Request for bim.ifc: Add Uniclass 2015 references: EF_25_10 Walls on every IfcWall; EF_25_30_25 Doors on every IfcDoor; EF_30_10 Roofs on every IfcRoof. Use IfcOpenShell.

First a look at what the model holds.

```python
import ifcopenshell

model = ifcopenshell.open("bim.ifc")
print(model.schema)
print("classifications:", [c.Name for c in model.by_type("IfcClassification")])
for ifc_class in ("IfcDoor", "IfcRoof", "IfcStair", "IfcWall", "IfcWindow"):
    print(ifc_class, len(model.by_type(ifc_class)))
```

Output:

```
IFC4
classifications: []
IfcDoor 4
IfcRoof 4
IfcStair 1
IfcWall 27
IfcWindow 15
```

```python
import ifcopenshell
import ifcopenshell.api.classification

model = ifcopenshell.open("bim.ifc")

system = ifcopenshell.api.classification.add_classification(model, classification="Uniclass 2015")

codes = {
    "IfcWall": ("EF_25_10", "Walls"),
    "IfcDoor": ("EF_25_30_25", "Doors"),
    "IfcRoof": ("EF_30_10", "Roofs"),
}
for ifc_class, (code, name) in codes.items():
    products = model.by_type(ifc_class)
    ifcopenshell.api.classification.add_reference(
        model, products=products, classification=system, identification=code, name=name
    )
    print(code, len(products))

model.write("bim-out.ifc")
```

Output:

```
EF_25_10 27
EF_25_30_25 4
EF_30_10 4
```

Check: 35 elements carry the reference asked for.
